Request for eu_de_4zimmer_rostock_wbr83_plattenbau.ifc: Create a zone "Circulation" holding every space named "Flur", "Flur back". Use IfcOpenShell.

First a look at what the model holds.

```python
import ifcopenshell

model = ifcopenshell.open("eu_de_4zimmer_rostock_wbr83_plattenbau.ifc")
print(model.schema)
seen = {}
for space in model.by_type("IfcSpace"):
    seen[space.LongName] = seen.get(space.LongName, 0) + 1
for name, count in sorted(seen.items(), key=str):
    print(count, "x", name)
print("zones:", [z.Name for z in model.by_type("IfcZone")][:20])
```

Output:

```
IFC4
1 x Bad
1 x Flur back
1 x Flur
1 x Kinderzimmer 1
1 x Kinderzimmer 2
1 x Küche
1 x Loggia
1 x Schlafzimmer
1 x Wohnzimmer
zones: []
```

```python
import ifcopenshell
import ifcopenshell.api.group
import ifcopenshell.api.root

model = ifcopenshell.open("eu_de_4zimmer_rostock_wbr83_plattenbau.ifc")

names = {"Flur", "Flur back"}
spaces = [s for s in model.by_type("IfcSpace") if s.LongName in names]

zone = ifcopenshell.api.root.create_entity(model, ifc_class="IfcZone", name="Circulation")
ifcopenshell.api.group.assign_group(model, products=spaces, group=zone)
print(len(spaces), "spaces in", zone.Name)

model.write("eu_de_4zimmer_rostock_wbr83_plattenbau_updated.ifc")
```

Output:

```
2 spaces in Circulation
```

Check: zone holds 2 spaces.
